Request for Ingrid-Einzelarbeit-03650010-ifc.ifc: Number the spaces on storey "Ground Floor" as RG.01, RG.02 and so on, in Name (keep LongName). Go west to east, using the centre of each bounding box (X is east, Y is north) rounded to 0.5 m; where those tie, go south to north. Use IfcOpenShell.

First a look at what the model holds.

```python
import ifcopenshell
import ifcopenshell.util.element
import ifcopenshell.util.placement

model = ifcopenshell.open("Ingrid-Einzelarbeit-03650010-ifc.ifc")
print(model.schema)
storey = next(s for s in model.by_type("IfcBuildingStorey") if s.Name == "Ground Floor")
spaces = [e for e in ifcopenshell.util.element.get_decomposition(storey) if e.is_a("IfcSpace")]
for e in sorted(spaces, key=lambda e: e.id()):
    origin = ifcopenshell.util.placement.get_local_placement(e.ObjectPlacement)[:3, 3]
    print(e.id(), e.Name, e.LongName, origin.round(2) + 0.0, sep=" | ")
```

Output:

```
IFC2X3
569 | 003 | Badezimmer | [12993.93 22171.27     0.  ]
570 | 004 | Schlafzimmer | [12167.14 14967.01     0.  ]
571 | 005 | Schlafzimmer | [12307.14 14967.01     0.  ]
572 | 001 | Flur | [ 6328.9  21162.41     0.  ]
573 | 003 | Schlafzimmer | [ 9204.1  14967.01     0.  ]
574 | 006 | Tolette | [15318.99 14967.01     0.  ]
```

```python
import ifcopenshell
import ifcopenshell.geom
import ifcopenshell.util.element
import ifcopenshell.util.shape

model = ifcopenshell.open("Ingrid-Einzelarbeit-03650010-ifc.ifc")
settings = ifcopenshell.geom.settings()
settings.set("use-world-coords", True)


def centre(element):
    shape = ifcopenshell.geom.create_shape(settings, element)
    return ifcopenshell.util.shape.get_bbox_centroid(shape.geometry)


storey = next(s for s in model.by_type("IfcBuildingStorey") if s.Name == "Ground Floor")
spaces = [e for e in ifcopenshell.util.element.get_decomposition(storey) if e.is_a("IfcSpace")]

# Insertion points can sit at a corner or the storey origin, so sort by the geometry (in metres).
centres = {e: centre(e) for e in spaces}
spaces.sort(key=lambda e: (round(centres[e][0] / 0.5), centres[e][1]))

for i, e in enumerate(spaces, start=1):
    number = f"RG.{i:02d}"
    e.Name = number
    print(e.id(), number)

model.write("Ingrid-Einzelarbeit-03650010-ifc_updated.ifc")
```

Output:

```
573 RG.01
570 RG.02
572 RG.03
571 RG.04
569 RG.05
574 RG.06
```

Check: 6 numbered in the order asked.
